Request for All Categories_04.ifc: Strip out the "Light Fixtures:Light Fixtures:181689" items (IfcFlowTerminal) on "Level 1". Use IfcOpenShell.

First a look at what the model holds.

```python
import ifcopenshell
import ifcopenshell.util.element

model = ifcopenshell.open("All Categories_04.ifc")
print(model.schema)
storey = next(s for s in model.by_type("IfcBuildingStorey") if s.Name == "Level 1")
terminals = [e for e in ifcopenshell.util.element.get_decomposition(storey) if e.is_a("IfcFlowTerminal")]
seen = {}
for e in terminals:
    element_type = ifcopenshell.util.element.get_type(e)
    name = element_type.Name if element_type not in (None, e) else None
    seen[name] = seen.get(name, 0) + 1
for name, count in sorted(seen.items(), key=str):
    print(count, "x", name)
```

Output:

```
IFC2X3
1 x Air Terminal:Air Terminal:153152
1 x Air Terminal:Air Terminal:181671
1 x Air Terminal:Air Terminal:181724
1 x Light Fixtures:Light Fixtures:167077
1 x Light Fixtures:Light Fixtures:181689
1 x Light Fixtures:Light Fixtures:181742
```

```python
import ifcopenshell
import ifcopenshell.api.root
import ifcopenshell.util.element

model = ifcopenshell.open("All Categories_04.ifc")

storey = next(s for s in model.by_type("IfcBuildingStorey") if s.Name == "Level 1")
terminals = [e for e in ifcopenshell.util.element.get_decomposition(storey) if e.is_a("IfcFlowTerminal")]
targets = [e for e in terminals if (t := ifcopenshell.util.element.get_type(e)) not in (None, e) and t.Name == "Light Fixtures:Light Fixtures:181689"]

for e in targets:
    ifcopenshell.api.root.remove_product(model, product=e)
print(len(targets), "removed")

model.write("All Categories_04_edited.ifc")
```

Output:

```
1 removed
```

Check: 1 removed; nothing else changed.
